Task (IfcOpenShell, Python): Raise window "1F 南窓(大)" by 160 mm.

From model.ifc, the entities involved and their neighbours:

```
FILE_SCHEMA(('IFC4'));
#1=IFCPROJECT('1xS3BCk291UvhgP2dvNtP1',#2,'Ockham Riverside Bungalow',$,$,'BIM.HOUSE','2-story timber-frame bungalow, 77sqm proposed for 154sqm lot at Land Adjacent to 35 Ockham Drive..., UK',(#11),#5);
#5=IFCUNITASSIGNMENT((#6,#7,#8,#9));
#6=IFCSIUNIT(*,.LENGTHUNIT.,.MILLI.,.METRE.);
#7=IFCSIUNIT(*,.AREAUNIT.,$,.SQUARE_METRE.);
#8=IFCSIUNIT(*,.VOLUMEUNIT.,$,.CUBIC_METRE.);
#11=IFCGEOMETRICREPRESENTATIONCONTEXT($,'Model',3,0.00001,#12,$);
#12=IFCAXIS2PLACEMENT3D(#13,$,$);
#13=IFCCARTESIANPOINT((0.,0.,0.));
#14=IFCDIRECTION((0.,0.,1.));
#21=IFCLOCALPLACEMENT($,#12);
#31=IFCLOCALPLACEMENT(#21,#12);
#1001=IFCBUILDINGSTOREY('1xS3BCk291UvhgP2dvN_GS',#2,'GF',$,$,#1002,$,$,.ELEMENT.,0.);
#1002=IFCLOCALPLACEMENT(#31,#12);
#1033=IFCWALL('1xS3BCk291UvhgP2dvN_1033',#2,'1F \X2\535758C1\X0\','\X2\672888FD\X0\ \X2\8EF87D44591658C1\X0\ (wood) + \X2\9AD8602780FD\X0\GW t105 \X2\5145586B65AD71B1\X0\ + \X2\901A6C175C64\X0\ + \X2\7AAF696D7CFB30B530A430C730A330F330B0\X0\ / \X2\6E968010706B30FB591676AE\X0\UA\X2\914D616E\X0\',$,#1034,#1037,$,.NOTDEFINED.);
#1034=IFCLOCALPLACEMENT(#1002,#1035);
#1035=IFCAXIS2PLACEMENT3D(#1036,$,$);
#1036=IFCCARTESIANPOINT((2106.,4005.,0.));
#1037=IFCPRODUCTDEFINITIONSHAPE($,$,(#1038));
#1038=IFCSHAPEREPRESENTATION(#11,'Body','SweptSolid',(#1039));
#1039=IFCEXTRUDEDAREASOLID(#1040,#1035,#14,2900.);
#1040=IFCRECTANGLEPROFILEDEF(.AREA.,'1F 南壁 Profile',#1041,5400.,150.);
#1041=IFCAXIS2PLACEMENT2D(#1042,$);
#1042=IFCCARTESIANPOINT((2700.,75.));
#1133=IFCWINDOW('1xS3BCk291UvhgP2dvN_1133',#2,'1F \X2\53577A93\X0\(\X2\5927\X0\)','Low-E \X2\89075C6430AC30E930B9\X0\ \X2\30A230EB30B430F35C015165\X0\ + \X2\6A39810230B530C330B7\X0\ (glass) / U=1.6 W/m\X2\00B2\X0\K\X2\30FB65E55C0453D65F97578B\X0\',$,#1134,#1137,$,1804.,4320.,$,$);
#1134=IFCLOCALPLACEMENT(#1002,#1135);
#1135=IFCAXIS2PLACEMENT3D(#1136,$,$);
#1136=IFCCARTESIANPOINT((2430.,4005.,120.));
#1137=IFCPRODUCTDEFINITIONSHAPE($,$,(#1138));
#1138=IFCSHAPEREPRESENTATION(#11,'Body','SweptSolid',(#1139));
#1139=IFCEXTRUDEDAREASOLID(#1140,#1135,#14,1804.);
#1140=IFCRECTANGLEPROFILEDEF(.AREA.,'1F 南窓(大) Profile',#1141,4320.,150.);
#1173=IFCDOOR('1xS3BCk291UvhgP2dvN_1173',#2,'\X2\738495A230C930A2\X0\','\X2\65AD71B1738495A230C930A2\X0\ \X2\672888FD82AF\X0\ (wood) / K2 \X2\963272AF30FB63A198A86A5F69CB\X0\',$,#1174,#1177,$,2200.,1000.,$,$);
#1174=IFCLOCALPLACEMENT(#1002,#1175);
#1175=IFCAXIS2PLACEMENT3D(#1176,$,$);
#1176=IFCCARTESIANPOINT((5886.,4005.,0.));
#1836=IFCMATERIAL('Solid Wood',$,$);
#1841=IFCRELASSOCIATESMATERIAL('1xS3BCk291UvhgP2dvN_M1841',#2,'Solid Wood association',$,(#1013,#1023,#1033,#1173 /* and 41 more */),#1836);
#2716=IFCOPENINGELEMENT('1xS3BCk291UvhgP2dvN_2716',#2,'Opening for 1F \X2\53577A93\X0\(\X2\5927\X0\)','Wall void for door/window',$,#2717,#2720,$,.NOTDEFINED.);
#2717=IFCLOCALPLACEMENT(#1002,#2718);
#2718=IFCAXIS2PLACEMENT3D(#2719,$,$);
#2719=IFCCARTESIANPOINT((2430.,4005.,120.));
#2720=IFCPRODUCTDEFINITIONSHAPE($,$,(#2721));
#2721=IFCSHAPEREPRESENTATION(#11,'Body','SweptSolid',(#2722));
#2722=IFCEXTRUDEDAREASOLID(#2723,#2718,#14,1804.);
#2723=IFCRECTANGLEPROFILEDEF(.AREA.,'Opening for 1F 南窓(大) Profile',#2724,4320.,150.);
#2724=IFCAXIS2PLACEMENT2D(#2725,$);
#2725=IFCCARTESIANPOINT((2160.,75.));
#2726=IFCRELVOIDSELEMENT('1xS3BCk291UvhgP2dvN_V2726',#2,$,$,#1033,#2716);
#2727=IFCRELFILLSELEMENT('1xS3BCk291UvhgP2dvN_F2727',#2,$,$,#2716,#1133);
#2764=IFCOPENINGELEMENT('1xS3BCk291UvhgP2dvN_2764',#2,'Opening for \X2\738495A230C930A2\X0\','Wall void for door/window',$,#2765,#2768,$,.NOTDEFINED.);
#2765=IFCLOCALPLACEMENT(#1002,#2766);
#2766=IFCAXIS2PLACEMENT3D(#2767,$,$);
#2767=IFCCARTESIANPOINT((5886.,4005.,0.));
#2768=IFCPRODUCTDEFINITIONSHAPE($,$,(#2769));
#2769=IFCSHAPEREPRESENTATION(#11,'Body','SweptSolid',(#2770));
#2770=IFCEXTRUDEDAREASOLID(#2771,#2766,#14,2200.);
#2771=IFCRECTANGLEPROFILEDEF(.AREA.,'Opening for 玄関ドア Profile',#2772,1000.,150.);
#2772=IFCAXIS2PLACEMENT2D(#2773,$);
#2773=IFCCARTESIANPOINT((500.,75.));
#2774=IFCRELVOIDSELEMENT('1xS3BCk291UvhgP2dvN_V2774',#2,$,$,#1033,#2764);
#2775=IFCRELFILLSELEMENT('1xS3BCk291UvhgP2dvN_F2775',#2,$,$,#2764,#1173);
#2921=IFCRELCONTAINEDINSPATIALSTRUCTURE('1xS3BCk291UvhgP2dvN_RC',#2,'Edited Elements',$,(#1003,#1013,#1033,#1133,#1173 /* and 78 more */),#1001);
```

```python
import numpy as np
import ifcopenshell
import ifcopenshell.api.geometry
import ifcopenshell.util.placement
import ifcopenshell.util.unit

model = ifcopenshell.open("model.ifc")
unit_scale = ifcopenshell.util.unit.calculate_unit_scale(model)

window = model.by_guid("1xS3BCk291UvhgP2dvN_1133")
opening = window.FillsVoids[0].RelatingOpeningElement
dz = 0.16 / unit_scale

shift = np.array([0.0, 0.0, dz])
# The window is not placed relative to its opening, so move both.
for product in (opening, window):
    matrix = ifcopenshell.util.placement.get_local_placement(product.ObjectPlacement)
    matrix[:3, 3] += shift
    ifcopenshell.api.geometry.edit_object_placement(model, product=product, matrix=matrix, is_si=False)

print(f"moved by {dz * unit_scale:+.3f} m")

model.write("model_edited.ifc")
```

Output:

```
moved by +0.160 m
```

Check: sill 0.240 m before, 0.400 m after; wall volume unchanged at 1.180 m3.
